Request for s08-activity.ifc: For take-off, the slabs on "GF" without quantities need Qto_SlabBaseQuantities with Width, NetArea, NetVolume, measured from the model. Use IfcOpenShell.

First a look at what the model holds.

```python
import ifcopenshell
import ifcopenshell.util.element
import ifcopenshell.util.unit

model = ifcopenshell.open("s08-activity.ifc")
print(model.schema)
for unit_type in ("LENGTHUNIT", "AREAUNIT", "VOLUMEUNIT"):
    print(unit_type, ifcopenshell.util.unit.calculate_unit_scale(model, unit_type))
storey = next(s for s in model.by_type("IfcBuildingStorey") if s.Name == "GF")
slabs = [e for e in ifcopenshell.util.element.get_decomposition(storey) if e.is_a("IfcSlab")]
for e in sorted(slabs, key=lambda e: e.id()):
    print(e.id(), e.is_a(), e.Name, list(ifcopenshell.util.element.get_psets(e, qtos_only=True)), sep=" | ")
```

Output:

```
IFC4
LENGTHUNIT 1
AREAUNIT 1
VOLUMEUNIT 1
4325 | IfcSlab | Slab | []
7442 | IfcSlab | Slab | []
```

```python
import ifcopenshell
import ifcopenshell.api.pset
import ifcopenshell.geom
import ifcopenshell.util.element
import ifcopenshell.util.shape
import ifcopenshell.util.unit

model = ifcopenshell.open("s08-activity.ifc")
unit_scale = ifcopenshell.util.unit.calculate_unit_scale(model)
area_scale = ifcopenshell.util.unit.calculate_unit_scale(model, "AREAUNIT")
volume_scale = ifcopenshell.util.unit.calculate_unit_scale(model, "VOLUMEUNIT")
settings = ifcopenshell.geom.settings()

storey = next(s for s in model.by_type("IfcBuildingStorey") if s.Name == "GF")
slabs = [e for e in ifcopenshell.util.element.get_decomposition(storey) if e.is_a("IfcSlab")]

for e in sorted(slabs, key=lambda e: e.id()):
    if ifcopenshell.util.element.get_psets(e, qtos_only=True, should_inherit=False):
        continue
    # Geometry comes back in metres, in the element's own axes.
    shape = ifcopenshell.geom.create_shape(settings, e)
    values = {
        "Width": ifcopenshell.util.shape.get_z(shape.geometry) / unit_scale,
        "NetArea": ifcopenshell.util.shape.get_footprint_area(shape.geometry) / area_scale,
        "NetVolume": ifcopenshell.util.shape.get_volume(shape.geometry) / volume_scale,
    }
    qto = ifcopenshell.api.pset.add_qto(model, product=e, name="Qto_SlabBaseQuantities")
    ifcopenshell.api.pset.edit_qto(model, qto=qto, properties=values)
    print(e.id(), {k: round(v, 3) for k, v in values.items()})

model.write("s08-activity_updated.ifc")
```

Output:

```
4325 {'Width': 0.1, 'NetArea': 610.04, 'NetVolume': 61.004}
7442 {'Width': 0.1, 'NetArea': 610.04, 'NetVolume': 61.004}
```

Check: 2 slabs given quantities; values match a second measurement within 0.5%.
